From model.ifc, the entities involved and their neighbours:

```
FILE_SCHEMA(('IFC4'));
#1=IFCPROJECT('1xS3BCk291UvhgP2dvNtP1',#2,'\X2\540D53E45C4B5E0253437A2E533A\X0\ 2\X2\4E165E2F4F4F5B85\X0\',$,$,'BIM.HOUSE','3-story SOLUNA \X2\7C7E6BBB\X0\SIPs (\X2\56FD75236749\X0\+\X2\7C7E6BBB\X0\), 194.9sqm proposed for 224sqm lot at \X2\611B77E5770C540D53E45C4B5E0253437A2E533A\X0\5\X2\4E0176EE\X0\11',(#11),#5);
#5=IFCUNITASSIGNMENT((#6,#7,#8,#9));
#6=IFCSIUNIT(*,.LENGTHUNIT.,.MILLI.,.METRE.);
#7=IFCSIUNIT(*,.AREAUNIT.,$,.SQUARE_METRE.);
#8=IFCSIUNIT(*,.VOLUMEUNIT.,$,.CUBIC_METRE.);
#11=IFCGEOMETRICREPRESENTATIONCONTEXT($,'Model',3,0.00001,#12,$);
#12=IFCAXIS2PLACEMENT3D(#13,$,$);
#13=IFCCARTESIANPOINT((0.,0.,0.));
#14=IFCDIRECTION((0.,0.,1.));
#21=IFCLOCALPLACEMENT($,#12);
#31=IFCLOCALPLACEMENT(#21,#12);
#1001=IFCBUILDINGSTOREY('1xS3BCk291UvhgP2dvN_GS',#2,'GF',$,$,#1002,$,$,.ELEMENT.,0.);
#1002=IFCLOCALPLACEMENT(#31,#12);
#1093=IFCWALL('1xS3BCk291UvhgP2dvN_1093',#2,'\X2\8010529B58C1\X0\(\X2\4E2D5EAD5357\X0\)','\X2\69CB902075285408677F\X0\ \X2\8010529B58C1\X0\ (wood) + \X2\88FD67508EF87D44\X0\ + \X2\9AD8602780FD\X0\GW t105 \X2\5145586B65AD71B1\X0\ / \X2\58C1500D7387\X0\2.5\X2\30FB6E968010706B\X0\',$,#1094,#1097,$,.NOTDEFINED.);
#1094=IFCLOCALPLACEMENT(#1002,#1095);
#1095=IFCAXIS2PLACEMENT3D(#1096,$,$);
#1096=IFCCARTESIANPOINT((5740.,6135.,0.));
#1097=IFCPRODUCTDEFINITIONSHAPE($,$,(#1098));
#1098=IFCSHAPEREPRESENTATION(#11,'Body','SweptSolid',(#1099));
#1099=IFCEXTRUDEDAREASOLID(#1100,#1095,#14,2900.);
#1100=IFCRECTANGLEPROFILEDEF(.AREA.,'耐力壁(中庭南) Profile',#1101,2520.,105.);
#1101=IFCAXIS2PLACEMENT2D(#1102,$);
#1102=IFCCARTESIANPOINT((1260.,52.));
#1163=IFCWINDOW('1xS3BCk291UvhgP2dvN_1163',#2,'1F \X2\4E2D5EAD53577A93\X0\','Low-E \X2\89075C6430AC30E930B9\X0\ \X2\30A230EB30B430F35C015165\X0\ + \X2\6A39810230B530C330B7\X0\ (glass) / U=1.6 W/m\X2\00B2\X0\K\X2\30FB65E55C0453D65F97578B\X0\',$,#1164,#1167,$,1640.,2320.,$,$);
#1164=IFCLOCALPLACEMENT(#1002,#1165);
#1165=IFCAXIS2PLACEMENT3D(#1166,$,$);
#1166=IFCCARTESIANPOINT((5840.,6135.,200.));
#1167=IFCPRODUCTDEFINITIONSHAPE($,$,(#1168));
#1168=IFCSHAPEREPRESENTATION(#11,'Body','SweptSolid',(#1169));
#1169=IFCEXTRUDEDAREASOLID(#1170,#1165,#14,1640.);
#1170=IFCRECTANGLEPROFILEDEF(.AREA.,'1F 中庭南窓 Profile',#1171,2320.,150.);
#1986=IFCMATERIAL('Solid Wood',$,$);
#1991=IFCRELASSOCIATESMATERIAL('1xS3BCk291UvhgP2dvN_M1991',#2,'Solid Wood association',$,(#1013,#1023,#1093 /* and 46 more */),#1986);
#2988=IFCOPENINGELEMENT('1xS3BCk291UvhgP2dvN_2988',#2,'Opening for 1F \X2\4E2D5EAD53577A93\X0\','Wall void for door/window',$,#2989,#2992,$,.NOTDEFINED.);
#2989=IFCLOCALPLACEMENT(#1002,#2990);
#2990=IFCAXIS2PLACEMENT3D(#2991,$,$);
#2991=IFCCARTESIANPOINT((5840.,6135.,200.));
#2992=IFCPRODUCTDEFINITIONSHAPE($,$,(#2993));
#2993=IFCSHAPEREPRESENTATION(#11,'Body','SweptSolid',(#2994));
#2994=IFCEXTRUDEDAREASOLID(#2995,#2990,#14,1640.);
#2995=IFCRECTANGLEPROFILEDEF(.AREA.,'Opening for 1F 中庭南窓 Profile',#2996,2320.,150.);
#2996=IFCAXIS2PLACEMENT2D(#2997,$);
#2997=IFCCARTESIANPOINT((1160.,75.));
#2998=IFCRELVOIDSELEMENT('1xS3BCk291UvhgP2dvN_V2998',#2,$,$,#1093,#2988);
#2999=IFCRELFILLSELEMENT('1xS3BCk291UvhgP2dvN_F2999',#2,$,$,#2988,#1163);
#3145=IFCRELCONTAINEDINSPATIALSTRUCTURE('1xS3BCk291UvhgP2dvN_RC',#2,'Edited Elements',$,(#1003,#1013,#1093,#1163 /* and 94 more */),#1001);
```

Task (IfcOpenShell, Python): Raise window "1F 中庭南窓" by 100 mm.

```python
import numpy as np
import ifcopenshell
import ifcopenshell.api.geometry
import ifcopenshell.util.placement
import ifcopenshell.util.unit

model = ifcopenshell.open("model.ifc")
unit_scale = ifcopenshell.util.unit.calculate_unit_scale(model)

window = model.by_guid("1xS3BCk291UvhgP2dvN_1163")
opening = window.FillsVoids[0].RelatingOpeningElement
dz = 100.0

shift = np.array([0.0, 0.0, dz])
# The window is not placed relative to its opening, so move both.
for product in (opening, window):
    matrix = ifcopenshell.util.placement.get_local_placement(product.ObjectPlacement)
    matrix[:3, 3] += shift
    ifcopenshell.api.geometry.edit_object_placement(model, product=product, matrix=matrix, is_si=False)

print(f"moved by {dz * unit_scale:+.3f} m")

model.write("model_updated.ifc")
```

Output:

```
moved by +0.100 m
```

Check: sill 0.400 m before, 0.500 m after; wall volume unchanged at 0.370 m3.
